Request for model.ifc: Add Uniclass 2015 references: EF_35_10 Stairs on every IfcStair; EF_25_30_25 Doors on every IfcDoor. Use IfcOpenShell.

First a look at what the model holds.

```python
import ifcopenshell

model = ifcopenshell.open("model.ifc")
print(model.schema)
print("classifications:", [c.Name for c in model.by_type("IfcClassification")])
for ifc_class in ("IfcDoor", "IfcRoof", "IfcStair", "IfcWall", "IfcWindow"):
    print(ifc_class, len(model.by_type(ifc_class)))
```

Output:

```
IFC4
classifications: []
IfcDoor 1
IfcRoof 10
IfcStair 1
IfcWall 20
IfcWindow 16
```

```python
import ifcopenshell
import ifcopenshell.api.classification

model = ifcopenshell.open("model.ifc")

system = ifcopenshell.api.classification.add_classification(model, classification="Uniclass 2015")

codes = {
    "IfcStair": ("EF_35_10", "Stairs"),
    "IfcDoor": ("EF_25_30_25", "Doors"),
}
for ifc_class, (code, name) in codes.items():
    products = model.by_type(ifc_class)
    ifcopenshell.api.classification.add_reference(
        model, products=products, classification=system, identification=code, name=name
    )
    print(code, len(products))

model.write("model_rev.ifc")
```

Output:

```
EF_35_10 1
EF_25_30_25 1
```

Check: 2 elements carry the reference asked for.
